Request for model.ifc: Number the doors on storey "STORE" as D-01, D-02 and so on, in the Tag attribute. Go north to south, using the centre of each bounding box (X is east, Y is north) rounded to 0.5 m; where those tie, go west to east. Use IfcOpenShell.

First a look at what the model holds.

```python
import ifcopenshell
import ifcopenshell.util.element
import ifcopenshell.util.placement

model = ifcopenshell.open("model.ifc")
print(model.schema)
storey = next(s for s in model.by_type("IfcBuildingStorey") if s.Name == "STORE")
doors = [e for e in ifcopenshell.util.element.get_decomposition(storey) if e.is_a("IfcDoor")]
for e in sorted(doors, key=lambda e: e.id()):
    origin = ifcopenshell.util.placement.get_local_placement(e.ObjectPlacement)[:3, 3]
    print(e.id(), e.Tag, e.Name, origin.round(2) + 0.0, sep=" | ")
```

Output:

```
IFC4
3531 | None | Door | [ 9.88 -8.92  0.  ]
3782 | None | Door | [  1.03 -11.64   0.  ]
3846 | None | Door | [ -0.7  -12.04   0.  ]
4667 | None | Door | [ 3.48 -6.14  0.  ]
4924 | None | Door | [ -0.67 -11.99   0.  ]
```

```python
import ifcopenshell
import ifcopenshell.geom
import ifcopenshell.util.element
import ifcopenshell.util.shape

model = ifcopenshell.open("model.ifc")
settings = ifcopenshell.geom.settings()
settings.set("use-world-coords", True)


def centre(element):
    shape = ifcopenshell.geom.create_shape(settings, element)
    return ifcopenshell.util.shape.get_bbox_centroid(shape.geometry)


storey = next(s for s in model.by_type("IfcBuildingStorey") if s.Name == "STORE")
doors = [e for e in ifcopenshell.util.element.get_decomposition(storey) if e.is_a("IfcDoor")]

# Insertion points can sit at a corner or the storey origin, so sort by the geometry (in metres).
centres = {e: centre(e) for e in doors}
doors.sort(key=lambda e: (-round(centres[e][1] / 0.5), centres[e][0]))

for i, e in enumerate(doors, start=1):
    number = f"D-{i:02d}"
    e.Tag = number
    print(e.id(), number)

model.write("model-out.ifc")
```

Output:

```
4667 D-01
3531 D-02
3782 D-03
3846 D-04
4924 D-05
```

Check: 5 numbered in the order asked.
